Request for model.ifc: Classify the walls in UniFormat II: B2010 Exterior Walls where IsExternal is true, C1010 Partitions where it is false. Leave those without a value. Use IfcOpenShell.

First a look at what the model holds.

```python
import ifcopenshell
import ifcopenshell.util.element

model = ifcopenshell.open("model.ifc")
print(model.schema)
print("classifications:", [c.Name for c in model.by_type("IfcClassification")])
values = [ifcopenshell.util.element.get_pset(e, "Pset_WallCommon", "IsExternal") for e in model.by_type("IfcWall")]
for value in (True, False, None):
    print("IsExternal", value, values.count(value))
```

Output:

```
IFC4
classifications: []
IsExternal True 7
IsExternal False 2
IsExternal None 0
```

```python
import ifcopenshell
import ifcopenshell.api.classification
import ifcopenshell.util.element

model = ifcopenshell.open("model.ifc")

system = ifcopenshell.api.classification.add_classification(model, classification="UniFormat II")

walls = model.by_type("IfcWall")
external = {e: ifcopenshell.util.element.get_pset(e, "Pset_WallCommon", "IsExternal") for e in walls}
for flag, code, name in ((True, "B2010", "Exterior Walls"), (False, "C1010", "Partitions")):
    products = [e for e in walls if external[e] is flag]
    ifcopenshell.api.classification.add_reference(
        model, products=products, classification=system, identification=code, name=name
    )
    print(code, len(products))

model.write("model_rev.ifc")
```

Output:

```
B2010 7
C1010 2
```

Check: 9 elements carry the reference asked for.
